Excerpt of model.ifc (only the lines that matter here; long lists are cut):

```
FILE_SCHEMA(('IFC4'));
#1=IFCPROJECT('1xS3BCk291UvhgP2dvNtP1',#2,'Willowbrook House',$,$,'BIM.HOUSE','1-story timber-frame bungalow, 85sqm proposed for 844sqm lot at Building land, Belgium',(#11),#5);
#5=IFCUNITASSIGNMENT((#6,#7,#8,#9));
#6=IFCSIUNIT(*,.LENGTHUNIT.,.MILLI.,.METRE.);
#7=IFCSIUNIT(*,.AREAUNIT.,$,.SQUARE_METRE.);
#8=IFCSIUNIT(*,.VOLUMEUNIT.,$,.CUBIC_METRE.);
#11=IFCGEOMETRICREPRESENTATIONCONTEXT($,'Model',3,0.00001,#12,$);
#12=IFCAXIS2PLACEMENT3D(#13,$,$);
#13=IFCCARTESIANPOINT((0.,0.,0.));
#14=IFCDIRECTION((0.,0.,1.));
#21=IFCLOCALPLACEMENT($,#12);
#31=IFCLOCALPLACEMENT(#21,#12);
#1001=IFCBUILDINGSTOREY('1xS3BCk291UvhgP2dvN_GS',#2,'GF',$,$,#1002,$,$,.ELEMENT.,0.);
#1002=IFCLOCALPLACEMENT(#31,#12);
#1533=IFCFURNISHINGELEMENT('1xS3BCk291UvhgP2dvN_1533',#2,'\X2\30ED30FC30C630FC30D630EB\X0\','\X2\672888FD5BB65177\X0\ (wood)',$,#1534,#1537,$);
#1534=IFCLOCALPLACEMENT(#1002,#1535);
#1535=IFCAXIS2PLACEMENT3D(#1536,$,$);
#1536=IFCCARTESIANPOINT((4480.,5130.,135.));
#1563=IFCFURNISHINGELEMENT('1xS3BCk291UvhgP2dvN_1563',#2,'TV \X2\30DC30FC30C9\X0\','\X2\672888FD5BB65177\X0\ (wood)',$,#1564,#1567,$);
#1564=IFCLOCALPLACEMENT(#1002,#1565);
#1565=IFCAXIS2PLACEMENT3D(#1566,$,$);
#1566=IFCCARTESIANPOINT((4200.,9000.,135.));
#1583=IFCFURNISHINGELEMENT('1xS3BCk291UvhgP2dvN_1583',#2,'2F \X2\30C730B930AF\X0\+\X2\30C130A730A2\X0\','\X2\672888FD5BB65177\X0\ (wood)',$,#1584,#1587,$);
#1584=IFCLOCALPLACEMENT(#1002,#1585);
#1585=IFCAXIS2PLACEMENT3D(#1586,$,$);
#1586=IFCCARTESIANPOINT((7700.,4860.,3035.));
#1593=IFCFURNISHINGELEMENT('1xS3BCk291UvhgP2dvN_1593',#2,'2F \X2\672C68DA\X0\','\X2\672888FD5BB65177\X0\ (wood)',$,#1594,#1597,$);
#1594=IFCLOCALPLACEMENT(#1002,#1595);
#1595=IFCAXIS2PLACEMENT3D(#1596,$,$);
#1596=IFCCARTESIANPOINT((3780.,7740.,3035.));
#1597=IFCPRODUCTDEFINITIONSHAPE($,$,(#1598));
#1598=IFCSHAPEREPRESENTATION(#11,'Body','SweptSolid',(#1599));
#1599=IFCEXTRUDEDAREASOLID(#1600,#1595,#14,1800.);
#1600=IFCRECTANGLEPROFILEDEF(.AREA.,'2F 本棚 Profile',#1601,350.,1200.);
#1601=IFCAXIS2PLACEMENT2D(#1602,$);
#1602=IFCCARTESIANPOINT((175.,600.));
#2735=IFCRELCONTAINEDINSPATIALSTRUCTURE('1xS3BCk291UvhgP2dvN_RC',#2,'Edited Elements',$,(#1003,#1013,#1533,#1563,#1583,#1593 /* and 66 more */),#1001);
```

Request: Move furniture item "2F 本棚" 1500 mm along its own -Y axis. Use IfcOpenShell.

```python
import ifcopenshell
import ifcopenshell.api.geometry
import ifcopenshell.util.placement
import ifcopenshell.util.unit

model = ifcopenshell.open("model.ifc")
unit_scale = ifcopenshell.util.unit.calculate_unit_scale(model)

item = model.by_id(1593)
matrix = ifcopenshell.util.placement.get_local_placement(item.ObjectPlacement)
matrix[:3, 3] -= matrix[:3, 1] * 1.5 / unit_scale
ifcopenshell.api.geometry.edit_object_placement(model, product=item, matrix=matrix, is_si=False)

print(ifcopenshell.util.placement.get_local_placement(item.ObjectPlacement).round(3) + 0.0)

model.write("model_updated.ifc")
```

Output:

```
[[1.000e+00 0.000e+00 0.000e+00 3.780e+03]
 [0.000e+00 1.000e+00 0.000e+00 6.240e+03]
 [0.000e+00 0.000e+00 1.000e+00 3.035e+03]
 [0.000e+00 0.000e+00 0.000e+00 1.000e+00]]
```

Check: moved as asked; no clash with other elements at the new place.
